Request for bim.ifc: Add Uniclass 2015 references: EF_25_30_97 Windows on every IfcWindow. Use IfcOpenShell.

First a look at what the model holds.

```python
import ifcopenshell

model = ifcopenshell.open("bim.ifc")
print(model.schema)
print("classifications:", [c.Name for c in model.by_type("IfcClassification")])
for ifc_class in ("IfcDoor", "IfcRoof", "IfcStair", "IfcWall", "IfcWindow"):
    print(ifc_class, len(model.by_type(ifc_class)))
```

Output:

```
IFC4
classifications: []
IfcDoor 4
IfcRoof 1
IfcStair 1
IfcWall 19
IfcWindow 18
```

```python
import ifcopenshell
import ifcopenshell.api.classification

model = ifcopenshell.open("bim.ifc")

system = ifcopenshell.api.classification.add_classification(model, classification="Uniclass 2015")

codes = {
    "IfcWindow": ("EF_25_30_97", "Windows"),
}
for ifc_class, (code, name) in codes.items():
    products = model.by_type(ifc_class)
    ifcopenshell.api.classification.add_reference(
        model, products=products, classification=system, identification=code, name=name
    )
    print(code, len(products))

model.write("bim_updated.ifc")
```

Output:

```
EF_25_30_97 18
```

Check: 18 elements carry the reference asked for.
